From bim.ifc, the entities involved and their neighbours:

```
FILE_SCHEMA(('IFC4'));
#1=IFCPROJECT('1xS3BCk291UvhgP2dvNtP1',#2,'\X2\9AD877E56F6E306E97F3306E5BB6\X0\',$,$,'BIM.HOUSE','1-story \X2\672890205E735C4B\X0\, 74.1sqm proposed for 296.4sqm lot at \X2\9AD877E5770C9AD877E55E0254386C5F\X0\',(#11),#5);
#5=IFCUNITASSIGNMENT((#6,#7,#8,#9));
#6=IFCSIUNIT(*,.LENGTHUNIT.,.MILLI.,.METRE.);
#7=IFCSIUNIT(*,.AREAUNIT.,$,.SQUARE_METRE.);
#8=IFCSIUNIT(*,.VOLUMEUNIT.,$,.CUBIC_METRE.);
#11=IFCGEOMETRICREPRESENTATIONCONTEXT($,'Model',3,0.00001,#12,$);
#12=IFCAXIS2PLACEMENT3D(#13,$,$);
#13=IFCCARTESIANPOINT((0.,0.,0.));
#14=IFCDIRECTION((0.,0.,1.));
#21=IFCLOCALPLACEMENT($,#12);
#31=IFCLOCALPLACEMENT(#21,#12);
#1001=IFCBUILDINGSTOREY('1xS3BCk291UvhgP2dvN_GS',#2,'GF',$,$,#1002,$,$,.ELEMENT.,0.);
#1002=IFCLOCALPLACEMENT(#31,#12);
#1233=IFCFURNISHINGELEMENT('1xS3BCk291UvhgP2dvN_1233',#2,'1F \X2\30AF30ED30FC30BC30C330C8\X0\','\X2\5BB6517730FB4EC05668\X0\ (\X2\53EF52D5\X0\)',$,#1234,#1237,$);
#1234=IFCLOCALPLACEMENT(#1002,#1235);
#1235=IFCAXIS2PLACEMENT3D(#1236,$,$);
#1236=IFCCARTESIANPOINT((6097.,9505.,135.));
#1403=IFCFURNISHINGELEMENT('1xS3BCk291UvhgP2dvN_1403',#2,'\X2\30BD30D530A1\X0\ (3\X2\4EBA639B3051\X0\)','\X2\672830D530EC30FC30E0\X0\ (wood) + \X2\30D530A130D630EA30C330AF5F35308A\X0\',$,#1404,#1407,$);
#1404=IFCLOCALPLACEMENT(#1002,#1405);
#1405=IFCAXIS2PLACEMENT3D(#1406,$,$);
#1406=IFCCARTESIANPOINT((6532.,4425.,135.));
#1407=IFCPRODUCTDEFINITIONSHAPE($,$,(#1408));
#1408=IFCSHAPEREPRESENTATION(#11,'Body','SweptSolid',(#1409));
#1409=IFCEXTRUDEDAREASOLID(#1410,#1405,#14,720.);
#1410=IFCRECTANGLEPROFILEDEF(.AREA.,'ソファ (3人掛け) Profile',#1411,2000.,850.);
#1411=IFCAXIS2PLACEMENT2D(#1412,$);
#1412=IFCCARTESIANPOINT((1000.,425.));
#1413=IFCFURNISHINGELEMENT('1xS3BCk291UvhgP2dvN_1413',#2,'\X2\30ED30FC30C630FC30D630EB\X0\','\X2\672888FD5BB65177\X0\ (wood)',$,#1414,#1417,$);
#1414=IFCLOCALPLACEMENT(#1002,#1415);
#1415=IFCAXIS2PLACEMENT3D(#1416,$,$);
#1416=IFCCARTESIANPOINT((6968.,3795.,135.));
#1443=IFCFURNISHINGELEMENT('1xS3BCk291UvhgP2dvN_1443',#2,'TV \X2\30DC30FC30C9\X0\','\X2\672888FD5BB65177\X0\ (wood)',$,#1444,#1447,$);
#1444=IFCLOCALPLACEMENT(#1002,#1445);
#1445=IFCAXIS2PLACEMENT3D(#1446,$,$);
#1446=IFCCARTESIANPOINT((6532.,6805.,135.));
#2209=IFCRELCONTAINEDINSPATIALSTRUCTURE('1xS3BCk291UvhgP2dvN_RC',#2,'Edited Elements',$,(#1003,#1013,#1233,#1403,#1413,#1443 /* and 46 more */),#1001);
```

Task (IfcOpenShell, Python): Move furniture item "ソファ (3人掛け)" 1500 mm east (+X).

```python
import ifcopenshell
import ifcopenshell.api.geometry
import ifcopenshell.util.placement

model = ifcopenshell.open("bim.ifc")

item = model.by_id(1403)
matrix = ifcopenshell.util.placement.get_local_placement(item.ObjectPlacement)
matrix[0, 3] += 1500.0
ifcopenshell.api.geometry.edit_object_placement(model, product=item, matrix=matrix, is_si=False)

print(ifcopenshell.util.placement.get_local_placement(item.ObjectPlacement).round(3) + 0.0)

model.write("bim-out.ifc")
```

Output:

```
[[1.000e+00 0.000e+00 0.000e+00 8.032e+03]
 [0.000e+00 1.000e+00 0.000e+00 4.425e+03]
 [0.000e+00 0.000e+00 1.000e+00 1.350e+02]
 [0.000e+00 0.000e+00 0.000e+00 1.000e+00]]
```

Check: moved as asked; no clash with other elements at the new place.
